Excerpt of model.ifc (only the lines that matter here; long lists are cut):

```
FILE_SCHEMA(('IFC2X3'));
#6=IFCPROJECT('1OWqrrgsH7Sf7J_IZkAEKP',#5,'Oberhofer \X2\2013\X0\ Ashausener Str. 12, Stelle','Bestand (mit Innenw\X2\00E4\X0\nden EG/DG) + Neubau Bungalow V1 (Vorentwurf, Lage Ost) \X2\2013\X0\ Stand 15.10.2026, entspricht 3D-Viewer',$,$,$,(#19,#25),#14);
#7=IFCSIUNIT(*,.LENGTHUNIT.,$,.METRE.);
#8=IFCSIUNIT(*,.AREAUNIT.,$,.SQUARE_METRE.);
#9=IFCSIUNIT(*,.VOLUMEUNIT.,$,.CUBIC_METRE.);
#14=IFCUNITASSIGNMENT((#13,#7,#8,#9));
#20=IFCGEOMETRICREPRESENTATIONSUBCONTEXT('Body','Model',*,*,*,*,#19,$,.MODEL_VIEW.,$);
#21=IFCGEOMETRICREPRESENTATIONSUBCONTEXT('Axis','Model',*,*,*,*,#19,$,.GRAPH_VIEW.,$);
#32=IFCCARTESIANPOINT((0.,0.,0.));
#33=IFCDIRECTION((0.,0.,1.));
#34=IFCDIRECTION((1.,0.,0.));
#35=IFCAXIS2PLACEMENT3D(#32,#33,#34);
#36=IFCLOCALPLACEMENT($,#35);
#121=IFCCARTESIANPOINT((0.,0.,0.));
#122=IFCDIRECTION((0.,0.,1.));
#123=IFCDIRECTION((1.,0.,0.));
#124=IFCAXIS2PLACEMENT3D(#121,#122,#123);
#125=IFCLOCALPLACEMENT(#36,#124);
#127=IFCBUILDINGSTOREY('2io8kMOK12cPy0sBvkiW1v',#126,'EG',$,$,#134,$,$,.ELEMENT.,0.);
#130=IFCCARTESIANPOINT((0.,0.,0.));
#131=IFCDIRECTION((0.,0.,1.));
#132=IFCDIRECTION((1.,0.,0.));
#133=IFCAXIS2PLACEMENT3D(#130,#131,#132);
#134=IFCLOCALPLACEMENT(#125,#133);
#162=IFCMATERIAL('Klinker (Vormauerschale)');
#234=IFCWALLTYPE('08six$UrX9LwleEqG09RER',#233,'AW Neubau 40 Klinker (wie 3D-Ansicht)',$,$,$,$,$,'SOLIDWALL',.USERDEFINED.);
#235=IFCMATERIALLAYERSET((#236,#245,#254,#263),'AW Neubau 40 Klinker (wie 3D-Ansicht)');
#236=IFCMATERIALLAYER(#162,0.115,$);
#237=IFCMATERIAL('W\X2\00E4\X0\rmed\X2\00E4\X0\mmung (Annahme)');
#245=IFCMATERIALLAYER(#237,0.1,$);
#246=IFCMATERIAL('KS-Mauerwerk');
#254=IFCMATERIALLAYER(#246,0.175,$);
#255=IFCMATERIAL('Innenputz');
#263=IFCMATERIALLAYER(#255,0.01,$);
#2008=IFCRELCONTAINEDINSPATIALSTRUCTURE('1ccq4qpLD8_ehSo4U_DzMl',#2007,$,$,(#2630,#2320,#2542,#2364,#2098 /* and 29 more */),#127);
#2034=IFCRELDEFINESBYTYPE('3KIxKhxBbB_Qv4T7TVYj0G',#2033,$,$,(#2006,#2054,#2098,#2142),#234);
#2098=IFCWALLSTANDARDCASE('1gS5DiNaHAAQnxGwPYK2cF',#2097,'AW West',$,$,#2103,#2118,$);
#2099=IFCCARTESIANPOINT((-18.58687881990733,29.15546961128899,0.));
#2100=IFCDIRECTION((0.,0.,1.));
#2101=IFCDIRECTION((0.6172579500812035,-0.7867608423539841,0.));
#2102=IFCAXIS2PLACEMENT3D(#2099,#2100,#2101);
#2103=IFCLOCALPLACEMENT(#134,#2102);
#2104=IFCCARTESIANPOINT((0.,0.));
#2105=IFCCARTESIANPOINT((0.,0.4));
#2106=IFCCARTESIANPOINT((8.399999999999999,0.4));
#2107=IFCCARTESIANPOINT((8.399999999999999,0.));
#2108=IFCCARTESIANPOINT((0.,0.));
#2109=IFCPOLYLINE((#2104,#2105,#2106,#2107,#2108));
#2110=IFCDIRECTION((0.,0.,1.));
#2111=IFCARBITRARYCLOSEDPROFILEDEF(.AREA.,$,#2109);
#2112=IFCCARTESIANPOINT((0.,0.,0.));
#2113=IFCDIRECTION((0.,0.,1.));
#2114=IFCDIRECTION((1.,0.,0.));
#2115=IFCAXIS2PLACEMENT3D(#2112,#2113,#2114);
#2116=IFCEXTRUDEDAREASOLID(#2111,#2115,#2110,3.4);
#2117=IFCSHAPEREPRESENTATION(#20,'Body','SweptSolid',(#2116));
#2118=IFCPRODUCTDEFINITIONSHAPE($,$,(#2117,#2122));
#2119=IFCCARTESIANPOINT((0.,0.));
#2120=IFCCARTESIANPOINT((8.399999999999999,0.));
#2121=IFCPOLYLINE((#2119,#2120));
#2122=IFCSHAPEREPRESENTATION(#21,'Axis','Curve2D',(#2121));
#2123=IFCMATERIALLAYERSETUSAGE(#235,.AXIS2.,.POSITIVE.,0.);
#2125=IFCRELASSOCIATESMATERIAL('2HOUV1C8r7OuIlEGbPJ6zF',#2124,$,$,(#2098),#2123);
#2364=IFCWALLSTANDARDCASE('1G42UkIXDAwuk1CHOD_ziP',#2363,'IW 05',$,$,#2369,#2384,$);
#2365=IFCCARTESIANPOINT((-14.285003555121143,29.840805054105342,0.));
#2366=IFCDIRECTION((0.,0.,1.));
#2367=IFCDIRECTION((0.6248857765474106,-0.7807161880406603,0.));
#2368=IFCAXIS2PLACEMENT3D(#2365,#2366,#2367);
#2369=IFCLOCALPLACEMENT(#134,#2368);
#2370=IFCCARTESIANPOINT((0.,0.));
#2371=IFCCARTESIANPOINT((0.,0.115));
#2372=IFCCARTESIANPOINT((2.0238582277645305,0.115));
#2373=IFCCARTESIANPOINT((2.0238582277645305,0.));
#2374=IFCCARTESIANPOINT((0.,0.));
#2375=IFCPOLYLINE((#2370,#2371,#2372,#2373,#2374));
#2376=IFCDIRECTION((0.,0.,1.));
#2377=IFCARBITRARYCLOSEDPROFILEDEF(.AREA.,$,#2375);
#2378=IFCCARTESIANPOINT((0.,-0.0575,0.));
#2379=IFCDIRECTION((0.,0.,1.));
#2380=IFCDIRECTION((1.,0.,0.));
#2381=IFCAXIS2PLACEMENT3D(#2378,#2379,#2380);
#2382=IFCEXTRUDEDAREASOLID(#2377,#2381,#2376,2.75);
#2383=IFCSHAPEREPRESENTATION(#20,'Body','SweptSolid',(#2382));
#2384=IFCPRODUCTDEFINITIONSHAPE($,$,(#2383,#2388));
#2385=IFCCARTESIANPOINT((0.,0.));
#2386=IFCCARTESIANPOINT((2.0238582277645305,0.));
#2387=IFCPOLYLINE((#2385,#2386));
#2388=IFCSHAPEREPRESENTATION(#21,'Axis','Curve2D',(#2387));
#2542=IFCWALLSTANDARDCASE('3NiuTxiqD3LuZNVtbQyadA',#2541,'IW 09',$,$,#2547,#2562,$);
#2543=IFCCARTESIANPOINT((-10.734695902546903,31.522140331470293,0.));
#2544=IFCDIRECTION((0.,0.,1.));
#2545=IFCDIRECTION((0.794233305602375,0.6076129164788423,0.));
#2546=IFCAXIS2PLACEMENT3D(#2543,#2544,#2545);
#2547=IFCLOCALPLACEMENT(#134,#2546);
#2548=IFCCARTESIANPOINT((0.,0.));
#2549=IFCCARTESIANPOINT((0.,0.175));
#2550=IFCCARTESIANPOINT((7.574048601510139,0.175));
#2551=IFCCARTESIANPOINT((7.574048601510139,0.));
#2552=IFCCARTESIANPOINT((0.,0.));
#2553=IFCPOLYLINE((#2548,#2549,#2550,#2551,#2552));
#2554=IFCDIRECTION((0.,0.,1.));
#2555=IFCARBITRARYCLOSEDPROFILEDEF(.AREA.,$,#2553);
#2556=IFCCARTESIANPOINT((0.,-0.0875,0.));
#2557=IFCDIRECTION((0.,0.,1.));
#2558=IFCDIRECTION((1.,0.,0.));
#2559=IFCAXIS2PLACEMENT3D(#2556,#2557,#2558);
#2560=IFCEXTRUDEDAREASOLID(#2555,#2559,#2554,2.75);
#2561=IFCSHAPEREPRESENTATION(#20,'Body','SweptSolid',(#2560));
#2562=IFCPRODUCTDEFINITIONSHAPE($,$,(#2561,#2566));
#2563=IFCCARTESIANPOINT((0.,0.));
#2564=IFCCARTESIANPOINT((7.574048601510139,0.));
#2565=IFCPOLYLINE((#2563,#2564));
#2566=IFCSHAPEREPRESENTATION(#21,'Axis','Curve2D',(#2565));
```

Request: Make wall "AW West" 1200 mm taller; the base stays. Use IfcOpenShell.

```python
import ifcopenshell
import ifcopenshell.geom
import ifcopenshell.util.representation
import ifcopenshell.util.shape
import ifcopenshell.util.unit

model = ifcopenshell.open("model.ifc")
unit_scale = ifcopenshell.util.unit.calculate_unit_scale(model)
settings = ifcopenshell.geom.settings()


def volume(element):
    """Net volume in cubic metres, openings subtracted."""
    shape = ifcopenshell.geom.create_shape(settings, element)
    return ifcopenshell.util.shape.get_volume(shape.geometry)


wall = model.by_guid("1gS5DiNaHAAQnxGwPYK2cF")
before = volume(wall)

body = ifcopenshell.util.representation.get_representation(wall, "Model", "Body")
solid = body.Items[0]
old_height = solid.Depth
solid.Depth += 1.2 / unit_scale
after = volume(wall)

print(f"height {old_height:g} -> {solid.Depth:g}, volume {before:.3f} -> {after:.3f} m3")

model.write("model_rev.ifc")
```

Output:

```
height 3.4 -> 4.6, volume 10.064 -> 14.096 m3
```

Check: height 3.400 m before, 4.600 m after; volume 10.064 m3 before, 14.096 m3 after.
